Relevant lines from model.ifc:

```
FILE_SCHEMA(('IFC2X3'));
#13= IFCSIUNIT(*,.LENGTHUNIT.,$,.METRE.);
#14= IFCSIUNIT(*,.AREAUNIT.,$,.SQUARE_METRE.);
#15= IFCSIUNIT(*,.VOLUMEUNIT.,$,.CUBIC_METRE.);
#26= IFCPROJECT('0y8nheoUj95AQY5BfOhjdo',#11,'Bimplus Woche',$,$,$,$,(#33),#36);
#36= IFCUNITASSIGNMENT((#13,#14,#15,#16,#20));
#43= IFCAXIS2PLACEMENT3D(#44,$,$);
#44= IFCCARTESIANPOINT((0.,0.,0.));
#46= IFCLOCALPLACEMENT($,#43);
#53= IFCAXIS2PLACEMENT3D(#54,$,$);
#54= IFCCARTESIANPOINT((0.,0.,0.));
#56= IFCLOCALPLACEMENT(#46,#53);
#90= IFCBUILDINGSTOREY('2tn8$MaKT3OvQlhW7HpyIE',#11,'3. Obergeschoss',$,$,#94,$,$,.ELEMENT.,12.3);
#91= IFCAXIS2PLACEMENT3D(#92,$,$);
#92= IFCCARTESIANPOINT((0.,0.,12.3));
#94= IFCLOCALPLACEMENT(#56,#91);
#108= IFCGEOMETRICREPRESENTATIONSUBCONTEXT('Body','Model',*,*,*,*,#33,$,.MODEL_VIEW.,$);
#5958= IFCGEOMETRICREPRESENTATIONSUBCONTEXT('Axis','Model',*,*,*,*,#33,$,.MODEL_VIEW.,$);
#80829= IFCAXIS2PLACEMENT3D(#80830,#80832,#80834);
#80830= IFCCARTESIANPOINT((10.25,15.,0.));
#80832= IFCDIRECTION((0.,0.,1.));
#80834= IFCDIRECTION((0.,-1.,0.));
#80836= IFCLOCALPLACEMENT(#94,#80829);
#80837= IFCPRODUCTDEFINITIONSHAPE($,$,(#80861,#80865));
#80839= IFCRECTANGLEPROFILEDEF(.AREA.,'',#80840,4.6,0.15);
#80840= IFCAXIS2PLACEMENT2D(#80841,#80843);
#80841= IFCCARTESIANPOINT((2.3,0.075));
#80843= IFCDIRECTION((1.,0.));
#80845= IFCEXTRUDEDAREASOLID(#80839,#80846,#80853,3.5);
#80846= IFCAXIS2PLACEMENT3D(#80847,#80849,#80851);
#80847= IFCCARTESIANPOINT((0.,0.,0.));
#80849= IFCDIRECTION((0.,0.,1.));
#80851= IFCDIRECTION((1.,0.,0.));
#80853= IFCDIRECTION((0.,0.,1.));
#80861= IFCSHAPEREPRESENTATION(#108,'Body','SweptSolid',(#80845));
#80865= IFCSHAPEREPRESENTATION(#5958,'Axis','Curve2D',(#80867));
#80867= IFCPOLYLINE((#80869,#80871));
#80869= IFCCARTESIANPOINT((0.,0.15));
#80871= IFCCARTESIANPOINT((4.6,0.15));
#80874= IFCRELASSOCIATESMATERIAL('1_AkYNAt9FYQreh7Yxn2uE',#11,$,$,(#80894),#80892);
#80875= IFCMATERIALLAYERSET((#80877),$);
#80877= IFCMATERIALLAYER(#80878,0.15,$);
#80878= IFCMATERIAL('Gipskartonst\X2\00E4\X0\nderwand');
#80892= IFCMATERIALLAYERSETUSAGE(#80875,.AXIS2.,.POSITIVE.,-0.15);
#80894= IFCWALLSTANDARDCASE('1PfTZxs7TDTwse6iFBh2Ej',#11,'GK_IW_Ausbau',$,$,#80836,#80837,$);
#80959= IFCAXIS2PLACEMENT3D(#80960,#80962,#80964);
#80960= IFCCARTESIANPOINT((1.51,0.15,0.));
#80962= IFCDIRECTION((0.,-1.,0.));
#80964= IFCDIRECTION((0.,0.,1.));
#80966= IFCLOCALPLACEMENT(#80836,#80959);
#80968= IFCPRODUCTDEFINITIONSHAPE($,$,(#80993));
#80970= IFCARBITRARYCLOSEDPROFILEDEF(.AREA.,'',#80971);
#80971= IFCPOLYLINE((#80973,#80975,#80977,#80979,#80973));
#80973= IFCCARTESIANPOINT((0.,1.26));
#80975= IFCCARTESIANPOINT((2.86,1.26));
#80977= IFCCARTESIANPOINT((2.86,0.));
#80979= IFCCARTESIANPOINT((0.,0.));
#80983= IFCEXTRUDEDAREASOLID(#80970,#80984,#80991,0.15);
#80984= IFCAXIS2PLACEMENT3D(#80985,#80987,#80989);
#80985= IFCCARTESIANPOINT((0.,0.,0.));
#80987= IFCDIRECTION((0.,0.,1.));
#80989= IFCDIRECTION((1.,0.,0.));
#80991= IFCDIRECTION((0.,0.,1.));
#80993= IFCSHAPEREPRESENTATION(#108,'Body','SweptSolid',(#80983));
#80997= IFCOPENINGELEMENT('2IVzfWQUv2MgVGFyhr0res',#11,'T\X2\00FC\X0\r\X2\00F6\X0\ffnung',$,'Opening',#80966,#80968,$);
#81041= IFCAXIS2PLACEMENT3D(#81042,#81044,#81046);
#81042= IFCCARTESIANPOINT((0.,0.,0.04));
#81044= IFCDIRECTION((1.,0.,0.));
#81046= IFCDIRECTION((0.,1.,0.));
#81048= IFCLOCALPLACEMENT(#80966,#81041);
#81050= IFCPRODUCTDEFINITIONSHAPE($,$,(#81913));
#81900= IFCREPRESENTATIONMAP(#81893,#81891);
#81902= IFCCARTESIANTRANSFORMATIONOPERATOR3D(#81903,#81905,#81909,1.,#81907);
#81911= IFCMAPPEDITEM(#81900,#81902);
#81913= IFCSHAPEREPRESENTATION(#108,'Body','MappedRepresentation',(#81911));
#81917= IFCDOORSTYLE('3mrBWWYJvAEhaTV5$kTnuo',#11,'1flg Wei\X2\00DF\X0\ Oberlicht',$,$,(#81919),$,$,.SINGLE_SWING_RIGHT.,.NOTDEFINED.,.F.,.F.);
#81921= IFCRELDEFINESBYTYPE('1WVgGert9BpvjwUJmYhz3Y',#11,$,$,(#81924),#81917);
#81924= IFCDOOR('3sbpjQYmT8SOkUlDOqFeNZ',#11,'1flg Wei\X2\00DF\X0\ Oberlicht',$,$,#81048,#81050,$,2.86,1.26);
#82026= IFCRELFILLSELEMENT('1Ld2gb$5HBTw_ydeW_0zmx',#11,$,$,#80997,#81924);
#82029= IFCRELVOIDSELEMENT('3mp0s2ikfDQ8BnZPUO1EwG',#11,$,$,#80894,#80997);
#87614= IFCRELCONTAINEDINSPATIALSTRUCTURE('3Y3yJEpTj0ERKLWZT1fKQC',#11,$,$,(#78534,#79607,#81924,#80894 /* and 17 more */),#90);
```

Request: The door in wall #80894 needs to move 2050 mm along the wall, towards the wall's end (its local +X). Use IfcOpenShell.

```python
import ifcopenshell
import ifcopenshell.api.geometry
import ifcopenshell.util.placement

model = ifcopenshell.open("model.ifc")

door = model.by_guid("3sbpjQYmT8SOkUlDOqFeNZ")
opening = door.FillsVoids[0].RelatingOpeningElement
wall = opening.VoidsElements[0].RelatingBuildingElement

wall_matrix = ifcopenshell.util.placement.get_local_placement(wall.ObjectPlacement)
shift = wall_matrix[:3, 0] * 2.05
before = ifcopenshell.util.placement.get_local_placement(door.ObjectPlacement)[:3, 3].copy()

# The door is placed relative to its opening, so it follows when the opening moves.
matrix = ifcopenshell.util.placement.get_local_placement(opening.ObjectPlacement)
matrix[:3, 3] += shift
ifcopenshell.api.geometry.edit_object_placement(
    model, product=opening, matrix=matrix, is_si=False, should_transform_children=True
)

after = ifcopenshell.util.placement.get_local_placement(door.ObjectPlacement)[:3, 3]
print("door moved by", (after - before).round(3) + 0.0)

model.write("model_rev.ifc")
```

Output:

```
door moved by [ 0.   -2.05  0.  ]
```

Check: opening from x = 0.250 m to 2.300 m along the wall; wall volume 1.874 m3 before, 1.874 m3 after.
